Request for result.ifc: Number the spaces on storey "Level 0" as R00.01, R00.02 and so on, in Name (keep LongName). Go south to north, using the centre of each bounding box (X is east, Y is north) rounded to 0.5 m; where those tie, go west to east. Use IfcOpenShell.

First a look at what the model holds.

```python
import ifcopenshell
import ifcopenshell.util.element
import ifcopenshell.util.placement

model = ifcopenshell.open("result.ifc")
print(model.schema)
storey = next(s for s in model.by_type("IfcBuildingStorey") if s.Name == "Level 0")
spaces = [e for e in ifcopenshell.util.element.get_decomposition(storey) if e.is_a("IfcSpace")]
for e in sorted(spaces, key=lambda e: e.id()):
    origin = ifcopenshell.util.placement.get_local_placement(e.ObjectPlacement)[:3, 3]
    print(e.id(), e.Name, e.LongName, origin.round(2) + 0.0, sep=" | ")
```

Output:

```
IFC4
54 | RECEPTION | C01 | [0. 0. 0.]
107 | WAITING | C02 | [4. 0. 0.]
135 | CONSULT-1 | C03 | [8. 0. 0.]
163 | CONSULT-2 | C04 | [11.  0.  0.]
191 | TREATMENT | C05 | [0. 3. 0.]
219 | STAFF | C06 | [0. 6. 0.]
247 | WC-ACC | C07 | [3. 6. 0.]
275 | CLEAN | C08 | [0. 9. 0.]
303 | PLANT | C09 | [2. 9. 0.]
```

```python
import ifcopenshell
import ifcopenshell.geom
import ifcopenshell.util.element
import ifcopenshell.util.shape

model = ifcopenshell.open("result.ifc")
settings = ifcopenshell.geom.settings()
settings.set("use-world-coords", True)


def centre(element):
    shape = ifcopenshell.geom.create_shape(settings, element)
    return ifcopenshell.util.shape.get_bbox_centroid(shape.geometry)


storey = next(s for s in model.by_type("IfcBuildingStorey") if s.Name == "Level 0")
spaces = [e for e in ifcopenshell.util.element.get_decomposition(storey) if e.is_a("IfcSpace")]

# Insertion points can sit at a corner or the storey origin, so sort by the geometry (in metres).
centres = {e: centre(e) for e in spaces}
spaces.sort(key=lambda e: (round(centres[e][1] / 0.5), centres[e][0]))

for i, e in enumerate(spaces, start=1):
    number = f"R00.{i:02d}"
    e.Name = number
    print(e.id(), number)

model.write("result_rev.ifc")
```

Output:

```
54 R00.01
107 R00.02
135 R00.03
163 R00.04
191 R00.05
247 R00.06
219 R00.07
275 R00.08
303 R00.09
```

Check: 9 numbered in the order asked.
